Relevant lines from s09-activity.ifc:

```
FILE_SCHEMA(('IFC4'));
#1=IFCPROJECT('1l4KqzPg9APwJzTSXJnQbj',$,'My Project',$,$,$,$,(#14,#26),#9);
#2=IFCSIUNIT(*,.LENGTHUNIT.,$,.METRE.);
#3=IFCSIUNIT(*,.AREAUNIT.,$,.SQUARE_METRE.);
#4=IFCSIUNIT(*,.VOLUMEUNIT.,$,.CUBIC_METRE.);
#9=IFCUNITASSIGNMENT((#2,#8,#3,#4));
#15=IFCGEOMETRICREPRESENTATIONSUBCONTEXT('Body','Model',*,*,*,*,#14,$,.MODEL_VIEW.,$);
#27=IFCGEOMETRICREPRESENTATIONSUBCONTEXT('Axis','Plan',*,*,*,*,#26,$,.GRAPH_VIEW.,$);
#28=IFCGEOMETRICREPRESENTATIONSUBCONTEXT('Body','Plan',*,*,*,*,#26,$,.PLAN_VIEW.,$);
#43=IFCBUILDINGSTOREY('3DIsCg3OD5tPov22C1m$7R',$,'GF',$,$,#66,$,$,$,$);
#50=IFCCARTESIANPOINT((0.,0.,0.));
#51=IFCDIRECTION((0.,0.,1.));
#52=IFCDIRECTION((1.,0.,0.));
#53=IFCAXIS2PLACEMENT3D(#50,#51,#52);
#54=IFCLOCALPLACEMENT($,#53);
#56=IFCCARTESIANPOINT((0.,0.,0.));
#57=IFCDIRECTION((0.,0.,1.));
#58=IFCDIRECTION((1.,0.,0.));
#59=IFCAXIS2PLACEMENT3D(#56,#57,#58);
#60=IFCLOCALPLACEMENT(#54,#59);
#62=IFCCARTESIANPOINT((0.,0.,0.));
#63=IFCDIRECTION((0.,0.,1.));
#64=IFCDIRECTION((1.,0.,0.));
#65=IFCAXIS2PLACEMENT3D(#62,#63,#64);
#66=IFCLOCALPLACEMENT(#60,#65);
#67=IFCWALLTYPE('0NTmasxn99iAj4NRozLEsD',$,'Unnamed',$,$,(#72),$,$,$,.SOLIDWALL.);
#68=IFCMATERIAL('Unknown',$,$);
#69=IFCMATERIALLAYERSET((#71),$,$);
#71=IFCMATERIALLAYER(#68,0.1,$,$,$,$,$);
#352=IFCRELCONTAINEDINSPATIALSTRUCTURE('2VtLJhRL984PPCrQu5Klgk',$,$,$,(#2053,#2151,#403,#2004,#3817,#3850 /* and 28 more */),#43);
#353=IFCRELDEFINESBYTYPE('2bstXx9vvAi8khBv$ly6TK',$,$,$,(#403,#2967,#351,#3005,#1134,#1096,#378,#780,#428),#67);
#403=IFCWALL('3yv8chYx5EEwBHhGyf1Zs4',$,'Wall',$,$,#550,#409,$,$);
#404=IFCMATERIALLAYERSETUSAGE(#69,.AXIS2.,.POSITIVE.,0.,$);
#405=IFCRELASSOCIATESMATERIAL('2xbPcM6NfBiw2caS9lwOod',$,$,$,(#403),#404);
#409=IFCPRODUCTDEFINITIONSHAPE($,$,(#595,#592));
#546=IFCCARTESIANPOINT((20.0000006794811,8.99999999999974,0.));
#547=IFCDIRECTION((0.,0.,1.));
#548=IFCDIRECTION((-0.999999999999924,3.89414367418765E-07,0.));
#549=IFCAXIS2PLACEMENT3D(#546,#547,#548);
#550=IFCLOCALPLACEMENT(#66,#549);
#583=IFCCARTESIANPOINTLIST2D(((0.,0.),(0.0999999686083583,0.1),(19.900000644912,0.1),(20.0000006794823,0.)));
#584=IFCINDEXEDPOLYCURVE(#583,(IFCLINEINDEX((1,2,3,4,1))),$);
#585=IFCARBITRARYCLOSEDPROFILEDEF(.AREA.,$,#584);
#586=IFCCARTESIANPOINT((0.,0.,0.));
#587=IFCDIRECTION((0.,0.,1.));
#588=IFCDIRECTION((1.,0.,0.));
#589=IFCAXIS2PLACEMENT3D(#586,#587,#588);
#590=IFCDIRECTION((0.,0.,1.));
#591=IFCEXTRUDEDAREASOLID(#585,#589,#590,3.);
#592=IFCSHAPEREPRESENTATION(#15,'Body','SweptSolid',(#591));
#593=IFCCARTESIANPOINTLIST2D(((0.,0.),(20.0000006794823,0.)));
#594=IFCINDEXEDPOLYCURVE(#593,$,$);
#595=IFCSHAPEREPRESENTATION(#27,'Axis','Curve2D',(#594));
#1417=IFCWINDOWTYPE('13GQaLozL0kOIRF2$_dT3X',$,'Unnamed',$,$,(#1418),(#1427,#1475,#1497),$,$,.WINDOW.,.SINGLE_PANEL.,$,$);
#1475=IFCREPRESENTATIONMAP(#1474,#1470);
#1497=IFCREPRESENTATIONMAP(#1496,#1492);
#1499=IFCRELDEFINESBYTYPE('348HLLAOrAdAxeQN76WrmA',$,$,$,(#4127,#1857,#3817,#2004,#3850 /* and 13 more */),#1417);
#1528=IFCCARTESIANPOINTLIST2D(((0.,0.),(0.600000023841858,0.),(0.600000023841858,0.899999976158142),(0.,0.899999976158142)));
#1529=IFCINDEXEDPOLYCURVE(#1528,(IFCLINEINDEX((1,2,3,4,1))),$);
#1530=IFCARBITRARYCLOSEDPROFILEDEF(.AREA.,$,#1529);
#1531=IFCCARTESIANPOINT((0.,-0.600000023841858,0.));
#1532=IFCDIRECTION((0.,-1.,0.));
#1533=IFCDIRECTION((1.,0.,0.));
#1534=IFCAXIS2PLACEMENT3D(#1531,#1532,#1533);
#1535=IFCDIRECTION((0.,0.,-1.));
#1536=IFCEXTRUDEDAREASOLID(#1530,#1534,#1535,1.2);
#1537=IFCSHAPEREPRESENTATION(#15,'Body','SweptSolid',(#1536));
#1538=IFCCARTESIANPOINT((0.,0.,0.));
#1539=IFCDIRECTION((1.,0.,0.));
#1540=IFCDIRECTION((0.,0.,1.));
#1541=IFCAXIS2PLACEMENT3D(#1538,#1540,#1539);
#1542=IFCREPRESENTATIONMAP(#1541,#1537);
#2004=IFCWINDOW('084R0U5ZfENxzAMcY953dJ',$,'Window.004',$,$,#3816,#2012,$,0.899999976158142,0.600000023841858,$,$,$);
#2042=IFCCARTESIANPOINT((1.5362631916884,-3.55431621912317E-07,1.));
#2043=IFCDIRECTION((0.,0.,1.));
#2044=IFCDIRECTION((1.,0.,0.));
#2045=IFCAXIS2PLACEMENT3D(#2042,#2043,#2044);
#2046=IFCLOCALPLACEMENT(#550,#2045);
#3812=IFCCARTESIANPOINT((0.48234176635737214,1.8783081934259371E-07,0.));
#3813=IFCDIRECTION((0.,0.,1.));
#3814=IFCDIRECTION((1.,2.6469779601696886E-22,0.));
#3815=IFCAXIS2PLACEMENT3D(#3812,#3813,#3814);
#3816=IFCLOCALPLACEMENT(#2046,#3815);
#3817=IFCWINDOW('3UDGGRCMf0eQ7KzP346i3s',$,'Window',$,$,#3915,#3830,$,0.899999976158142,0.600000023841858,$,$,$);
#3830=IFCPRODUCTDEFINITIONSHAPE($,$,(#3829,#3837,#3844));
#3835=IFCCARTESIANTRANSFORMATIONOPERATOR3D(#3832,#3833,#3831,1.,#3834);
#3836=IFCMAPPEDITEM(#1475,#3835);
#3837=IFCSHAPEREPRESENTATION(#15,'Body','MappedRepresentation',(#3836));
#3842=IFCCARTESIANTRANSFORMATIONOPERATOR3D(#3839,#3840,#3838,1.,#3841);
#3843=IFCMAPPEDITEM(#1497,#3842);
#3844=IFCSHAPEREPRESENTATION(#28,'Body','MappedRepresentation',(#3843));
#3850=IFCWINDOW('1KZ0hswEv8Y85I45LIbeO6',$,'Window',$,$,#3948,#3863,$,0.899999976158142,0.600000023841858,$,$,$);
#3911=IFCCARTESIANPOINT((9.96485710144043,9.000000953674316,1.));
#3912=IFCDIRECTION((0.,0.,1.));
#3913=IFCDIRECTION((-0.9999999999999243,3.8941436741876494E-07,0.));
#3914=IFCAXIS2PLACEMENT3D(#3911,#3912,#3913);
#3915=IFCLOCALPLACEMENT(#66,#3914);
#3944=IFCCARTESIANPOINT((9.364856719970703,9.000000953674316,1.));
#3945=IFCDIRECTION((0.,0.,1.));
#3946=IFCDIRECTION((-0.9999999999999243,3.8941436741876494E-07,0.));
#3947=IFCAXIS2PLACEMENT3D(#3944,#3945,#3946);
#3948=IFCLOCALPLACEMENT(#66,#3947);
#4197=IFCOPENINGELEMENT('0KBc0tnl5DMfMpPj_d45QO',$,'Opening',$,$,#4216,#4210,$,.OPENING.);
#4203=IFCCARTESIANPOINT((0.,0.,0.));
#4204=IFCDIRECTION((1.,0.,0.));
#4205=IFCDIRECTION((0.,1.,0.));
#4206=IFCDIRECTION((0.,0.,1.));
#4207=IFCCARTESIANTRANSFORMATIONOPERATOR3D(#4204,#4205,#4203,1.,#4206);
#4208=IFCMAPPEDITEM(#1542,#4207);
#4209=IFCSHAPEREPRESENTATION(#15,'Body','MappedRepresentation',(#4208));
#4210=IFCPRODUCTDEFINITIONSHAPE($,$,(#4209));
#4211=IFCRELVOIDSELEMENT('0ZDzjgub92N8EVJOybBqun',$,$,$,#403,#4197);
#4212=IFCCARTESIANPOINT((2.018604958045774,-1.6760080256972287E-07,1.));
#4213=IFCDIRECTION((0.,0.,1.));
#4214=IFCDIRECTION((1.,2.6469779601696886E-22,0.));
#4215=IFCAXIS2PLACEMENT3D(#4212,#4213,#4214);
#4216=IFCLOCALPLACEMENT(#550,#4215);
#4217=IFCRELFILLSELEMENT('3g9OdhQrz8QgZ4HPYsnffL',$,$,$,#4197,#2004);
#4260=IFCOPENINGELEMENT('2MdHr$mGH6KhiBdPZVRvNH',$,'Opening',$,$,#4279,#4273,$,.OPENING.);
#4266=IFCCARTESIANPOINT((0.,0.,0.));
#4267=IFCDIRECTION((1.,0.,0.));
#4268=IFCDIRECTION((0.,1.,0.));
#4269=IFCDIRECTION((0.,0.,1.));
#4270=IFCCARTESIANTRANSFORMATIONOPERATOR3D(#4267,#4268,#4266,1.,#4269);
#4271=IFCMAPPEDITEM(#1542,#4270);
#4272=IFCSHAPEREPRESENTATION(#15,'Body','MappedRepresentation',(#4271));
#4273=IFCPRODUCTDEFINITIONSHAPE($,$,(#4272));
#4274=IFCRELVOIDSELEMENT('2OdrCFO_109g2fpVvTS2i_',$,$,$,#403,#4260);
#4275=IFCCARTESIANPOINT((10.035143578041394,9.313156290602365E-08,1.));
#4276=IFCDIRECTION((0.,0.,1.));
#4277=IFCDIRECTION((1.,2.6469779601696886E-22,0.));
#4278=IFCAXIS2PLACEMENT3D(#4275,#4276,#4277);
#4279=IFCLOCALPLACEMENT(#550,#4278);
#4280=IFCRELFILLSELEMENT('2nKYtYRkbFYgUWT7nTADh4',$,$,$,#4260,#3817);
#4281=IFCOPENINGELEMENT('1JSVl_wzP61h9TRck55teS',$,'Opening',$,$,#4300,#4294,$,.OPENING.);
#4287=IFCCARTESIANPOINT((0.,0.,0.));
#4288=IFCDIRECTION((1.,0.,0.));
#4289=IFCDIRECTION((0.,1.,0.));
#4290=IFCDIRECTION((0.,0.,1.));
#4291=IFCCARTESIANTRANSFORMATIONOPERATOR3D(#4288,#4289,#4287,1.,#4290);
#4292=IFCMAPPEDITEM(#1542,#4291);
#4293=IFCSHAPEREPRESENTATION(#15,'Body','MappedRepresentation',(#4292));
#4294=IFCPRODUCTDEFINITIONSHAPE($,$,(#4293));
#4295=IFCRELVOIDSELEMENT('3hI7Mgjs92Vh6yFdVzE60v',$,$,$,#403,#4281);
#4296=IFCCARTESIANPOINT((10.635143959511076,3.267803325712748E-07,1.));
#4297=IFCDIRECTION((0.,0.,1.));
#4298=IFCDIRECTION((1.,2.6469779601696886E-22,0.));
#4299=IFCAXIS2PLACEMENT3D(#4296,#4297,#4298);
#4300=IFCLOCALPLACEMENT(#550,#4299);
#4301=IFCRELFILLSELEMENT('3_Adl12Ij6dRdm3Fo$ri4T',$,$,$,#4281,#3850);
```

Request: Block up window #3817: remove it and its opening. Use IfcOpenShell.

```python
import ifcopenshell
import ifcopenshell.api.feature
import ifcopenshell.api.root
import ifcopenshell.geom
import ifcopenshell.util.shape

model = ifcopenshell.open("s09-activity.ifc")
settings = ifcopenshell.geom.settings()


def volume(element):
    """Net volume in cubic metres, openings subtracted."""
    shape = ifcopenshell.geom.create_shape(settings, element)
    return ifcopenshell.util.shape.get_volume(shape.geometry)


window = model.by_guid("3UDGGRCMf0eQ7KzP346i3s")
opening = window.FillsVoids[0].RelatingOpeningElement
wall = opening.VoidsElements[0].RelatingBuildingElement
before = volume(wall)

ifcopenshell.api.root.remove_product(model, product=window)
ifcopenshell.api.feature.remove_feature(model, feature=opening)

after = volume(wall)

print(f"wall volume {before:.3f} -> {after:.3f} m3")

model.write("s09-activity_updated.ifc")
```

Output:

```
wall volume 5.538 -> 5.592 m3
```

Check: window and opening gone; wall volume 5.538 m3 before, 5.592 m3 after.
